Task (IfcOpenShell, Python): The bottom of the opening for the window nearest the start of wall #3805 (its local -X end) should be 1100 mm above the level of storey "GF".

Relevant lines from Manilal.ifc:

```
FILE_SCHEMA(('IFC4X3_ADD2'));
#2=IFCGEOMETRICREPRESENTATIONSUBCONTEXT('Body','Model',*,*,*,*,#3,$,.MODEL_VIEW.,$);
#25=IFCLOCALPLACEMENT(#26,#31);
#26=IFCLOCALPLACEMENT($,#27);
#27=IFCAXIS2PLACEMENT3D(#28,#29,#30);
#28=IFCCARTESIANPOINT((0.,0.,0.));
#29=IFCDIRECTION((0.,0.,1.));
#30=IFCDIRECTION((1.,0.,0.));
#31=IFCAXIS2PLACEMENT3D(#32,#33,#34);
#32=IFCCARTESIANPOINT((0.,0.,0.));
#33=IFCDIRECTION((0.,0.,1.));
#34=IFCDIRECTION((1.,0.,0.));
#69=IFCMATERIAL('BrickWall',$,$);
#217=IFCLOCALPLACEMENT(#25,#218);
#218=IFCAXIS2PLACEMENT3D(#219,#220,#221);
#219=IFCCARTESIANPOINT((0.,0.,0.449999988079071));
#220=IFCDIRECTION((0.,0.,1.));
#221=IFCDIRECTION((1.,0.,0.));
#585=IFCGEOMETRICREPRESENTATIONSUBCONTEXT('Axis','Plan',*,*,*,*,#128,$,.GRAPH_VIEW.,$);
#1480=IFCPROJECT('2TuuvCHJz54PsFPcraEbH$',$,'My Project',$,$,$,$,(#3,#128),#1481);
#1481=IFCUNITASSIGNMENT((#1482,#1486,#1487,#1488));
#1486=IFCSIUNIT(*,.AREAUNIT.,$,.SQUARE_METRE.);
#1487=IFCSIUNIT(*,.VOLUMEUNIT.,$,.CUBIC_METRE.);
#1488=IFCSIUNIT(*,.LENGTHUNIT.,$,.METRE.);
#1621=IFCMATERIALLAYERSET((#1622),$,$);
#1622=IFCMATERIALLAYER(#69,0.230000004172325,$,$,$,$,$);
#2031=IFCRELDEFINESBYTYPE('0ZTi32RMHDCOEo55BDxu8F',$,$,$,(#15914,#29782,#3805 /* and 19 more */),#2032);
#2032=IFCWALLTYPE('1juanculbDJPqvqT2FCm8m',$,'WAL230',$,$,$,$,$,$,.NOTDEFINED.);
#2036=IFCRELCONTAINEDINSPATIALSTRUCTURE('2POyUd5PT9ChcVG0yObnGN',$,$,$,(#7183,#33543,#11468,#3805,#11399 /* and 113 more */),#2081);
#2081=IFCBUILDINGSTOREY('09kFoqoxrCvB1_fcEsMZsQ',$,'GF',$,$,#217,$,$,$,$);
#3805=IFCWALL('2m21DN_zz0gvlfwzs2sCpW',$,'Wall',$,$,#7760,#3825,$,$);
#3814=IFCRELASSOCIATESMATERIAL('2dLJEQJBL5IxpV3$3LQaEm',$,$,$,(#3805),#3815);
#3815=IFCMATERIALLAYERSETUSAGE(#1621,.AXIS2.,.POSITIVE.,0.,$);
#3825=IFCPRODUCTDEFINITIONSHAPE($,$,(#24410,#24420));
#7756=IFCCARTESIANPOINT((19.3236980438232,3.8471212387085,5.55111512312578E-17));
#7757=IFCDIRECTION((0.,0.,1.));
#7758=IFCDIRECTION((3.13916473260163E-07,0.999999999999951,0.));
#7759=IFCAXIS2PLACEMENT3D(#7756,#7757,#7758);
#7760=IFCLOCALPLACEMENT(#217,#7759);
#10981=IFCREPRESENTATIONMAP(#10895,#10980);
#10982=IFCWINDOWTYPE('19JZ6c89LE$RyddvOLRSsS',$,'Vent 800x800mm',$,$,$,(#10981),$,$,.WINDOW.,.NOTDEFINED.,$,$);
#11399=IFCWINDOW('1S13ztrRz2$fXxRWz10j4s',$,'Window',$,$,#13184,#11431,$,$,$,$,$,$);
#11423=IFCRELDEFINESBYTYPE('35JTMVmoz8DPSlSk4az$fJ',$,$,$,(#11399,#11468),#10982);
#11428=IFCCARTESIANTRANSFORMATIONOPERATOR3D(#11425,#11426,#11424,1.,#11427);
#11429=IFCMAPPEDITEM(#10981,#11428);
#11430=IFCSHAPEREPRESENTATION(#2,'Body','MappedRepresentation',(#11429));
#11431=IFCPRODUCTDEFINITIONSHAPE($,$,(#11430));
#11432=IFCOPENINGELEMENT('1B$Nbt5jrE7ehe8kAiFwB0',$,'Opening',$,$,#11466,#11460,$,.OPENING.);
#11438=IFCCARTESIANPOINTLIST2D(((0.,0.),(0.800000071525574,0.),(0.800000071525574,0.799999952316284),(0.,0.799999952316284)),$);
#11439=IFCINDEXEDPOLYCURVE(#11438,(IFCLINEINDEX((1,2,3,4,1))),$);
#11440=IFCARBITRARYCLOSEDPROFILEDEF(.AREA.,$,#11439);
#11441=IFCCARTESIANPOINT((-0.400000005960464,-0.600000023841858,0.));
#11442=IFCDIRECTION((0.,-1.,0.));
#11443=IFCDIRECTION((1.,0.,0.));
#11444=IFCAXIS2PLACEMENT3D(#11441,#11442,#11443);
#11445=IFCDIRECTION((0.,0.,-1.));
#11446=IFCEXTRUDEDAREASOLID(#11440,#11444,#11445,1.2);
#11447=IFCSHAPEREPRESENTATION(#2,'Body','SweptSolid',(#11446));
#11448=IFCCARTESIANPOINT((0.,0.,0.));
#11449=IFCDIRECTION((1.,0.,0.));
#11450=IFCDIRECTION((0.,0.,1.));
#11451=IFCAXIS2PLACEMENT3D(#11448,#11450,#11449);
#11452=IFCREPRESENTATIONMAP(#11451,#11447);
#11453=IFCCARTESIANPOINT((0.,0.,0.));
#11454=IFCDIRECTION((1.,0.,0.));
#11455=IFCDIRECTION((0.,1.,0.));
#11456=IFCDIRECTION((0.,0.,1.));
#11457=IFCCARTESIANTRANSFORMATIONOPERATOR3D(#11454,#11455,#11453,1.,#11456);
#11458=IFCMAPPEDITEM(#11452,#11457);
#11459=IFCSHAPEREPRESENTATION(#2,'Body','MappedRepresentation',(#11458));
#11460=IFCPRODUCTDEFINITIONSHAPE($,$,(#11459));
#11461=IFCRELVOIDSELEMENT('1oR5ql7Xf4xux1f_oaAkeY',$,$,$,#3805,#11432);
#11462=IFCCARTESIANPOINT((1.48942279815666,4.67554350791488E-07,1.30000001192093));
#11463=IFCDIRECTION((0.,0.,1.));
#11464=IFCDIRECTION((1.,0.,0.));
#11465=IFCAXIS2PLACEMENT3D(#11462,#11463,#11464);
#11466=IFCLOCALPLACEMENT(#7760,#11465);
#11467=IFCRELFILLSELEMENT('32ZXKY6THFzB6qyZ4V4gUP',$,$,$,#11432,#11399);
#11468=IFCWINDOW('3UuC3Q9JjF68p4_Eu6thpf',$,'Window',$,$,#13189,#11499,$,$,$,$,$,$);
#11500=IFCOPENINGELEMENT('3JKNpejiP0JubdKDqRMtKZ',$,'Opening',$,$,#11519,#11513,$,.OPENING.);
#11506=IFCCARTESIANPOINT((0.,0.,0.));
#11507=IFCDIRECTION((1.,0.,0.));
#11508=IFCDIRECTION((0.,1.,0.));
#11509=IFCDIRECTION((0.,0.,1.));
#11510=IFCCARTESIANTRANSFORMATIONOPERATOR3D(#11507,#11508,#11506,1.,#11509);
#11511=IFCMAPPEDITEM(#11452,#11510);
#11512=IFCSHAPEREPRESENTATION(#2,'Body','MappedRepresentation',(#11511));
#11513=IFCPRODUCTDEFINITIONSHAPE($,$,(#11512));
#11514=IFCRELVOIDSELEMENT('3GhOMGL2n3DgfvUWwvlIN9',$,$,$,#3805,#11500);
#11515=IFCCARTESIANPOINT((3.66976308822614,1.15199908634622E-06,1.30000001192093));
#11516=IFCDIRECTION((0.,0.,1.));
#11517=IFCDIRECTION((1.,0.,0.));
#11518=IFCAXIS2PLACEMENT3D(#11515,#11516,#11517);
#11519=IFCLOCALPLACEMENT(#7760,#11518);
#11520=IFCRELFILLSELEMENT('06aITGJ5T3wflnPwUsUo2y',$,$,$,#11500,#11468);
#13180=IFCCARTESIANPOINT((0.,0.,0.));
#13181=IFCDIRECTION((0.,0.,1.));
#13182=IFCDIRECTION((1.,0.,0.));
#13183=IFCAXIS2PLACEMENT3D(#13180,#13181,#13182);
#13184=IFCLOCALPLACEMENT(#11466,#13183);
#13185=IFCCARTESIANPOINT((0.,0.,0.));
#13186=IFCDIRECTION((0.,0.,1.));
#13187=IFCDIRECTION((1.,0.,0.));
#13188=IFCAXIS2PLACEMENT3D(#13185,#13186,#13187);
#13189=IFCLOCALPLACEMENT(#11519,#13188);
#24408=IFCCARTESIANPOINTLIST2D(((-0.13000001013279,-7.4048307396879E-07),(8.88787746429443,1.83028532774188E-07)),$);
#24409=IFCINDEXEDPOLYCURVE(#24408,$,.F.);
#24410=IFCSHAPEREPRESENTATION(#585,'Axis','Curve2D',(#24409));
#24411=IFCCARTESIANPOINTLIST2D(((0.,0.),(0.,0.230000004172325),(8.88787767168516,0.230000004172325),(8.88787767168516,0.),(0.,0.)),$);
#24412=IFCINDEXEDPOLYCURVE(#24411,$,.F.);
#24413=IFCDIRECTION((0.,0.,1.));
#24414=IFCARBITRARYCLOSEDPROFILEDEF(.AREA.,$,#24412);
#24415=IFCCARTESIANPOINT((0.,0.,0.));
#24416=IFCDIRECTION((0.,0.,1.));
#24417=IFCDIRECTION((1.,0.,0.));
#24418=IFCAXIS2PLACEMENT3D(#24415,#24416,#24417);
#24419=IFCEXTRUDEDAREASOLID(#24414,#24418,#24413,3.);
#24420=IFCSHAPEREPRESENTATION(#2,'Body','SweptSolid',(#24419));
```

```python
import numpy as np
import ifcopenshell
import ifcopenshell.api.geometry
import ifcopenshell.geom
import ifcopenshell.util.element
import ifcopenshell.util.placement
import ifcopenshell.util.shape
import ifcopenshell.util.unit

model = ifcopenshell.open("Manilal.ifc")
unit_scale = ifcopenshell.util.unit.calculate_unit_scale(model)

window = model.by_guid("1S13ztrRz2$fXxRWz10j4s")
opening = window.FillsVoids[0].RelatingOpeningElement
storey = ifcopenshell.util.element.get_container(window, ifc_class="IfcBuildingStorey")
level = ifcopenshell.util.placement.get_local_placement(storey.ObjectPlacement)[2, 3]

# The opening's origin need not be at the sill, so measure its lowest point.
shape = ifcopenshell.geom.create_shape(ifcopenshell.geom.settings(), opening)
bottom = ifcopenshell.util.shape.get_shape_bottom_elevation(shape, shape.geometry) / unit_scale
dz = level + 1.1 - bottom

shift = np.array([0.0, 0.0, dz])
# The window is placed relative to its opening, so it follows when the opening moves.
matrix = ifcopenshell.util.placement.get_local_placement(opening.ObjectPlacement)
matrix[:3, 3] += shift
ifcopenshell.api.geometry.edit_object_placement(
    model, product=opening, matrix=matrix, is_si=False, should_transform_children=True
)

print(f"moved by {dz * unit_scale:+.3f} m")

model.write("Manilal_rev.ifc")
```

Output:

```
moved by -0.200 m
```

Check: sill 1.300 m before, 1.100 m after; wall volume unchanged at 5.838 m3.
